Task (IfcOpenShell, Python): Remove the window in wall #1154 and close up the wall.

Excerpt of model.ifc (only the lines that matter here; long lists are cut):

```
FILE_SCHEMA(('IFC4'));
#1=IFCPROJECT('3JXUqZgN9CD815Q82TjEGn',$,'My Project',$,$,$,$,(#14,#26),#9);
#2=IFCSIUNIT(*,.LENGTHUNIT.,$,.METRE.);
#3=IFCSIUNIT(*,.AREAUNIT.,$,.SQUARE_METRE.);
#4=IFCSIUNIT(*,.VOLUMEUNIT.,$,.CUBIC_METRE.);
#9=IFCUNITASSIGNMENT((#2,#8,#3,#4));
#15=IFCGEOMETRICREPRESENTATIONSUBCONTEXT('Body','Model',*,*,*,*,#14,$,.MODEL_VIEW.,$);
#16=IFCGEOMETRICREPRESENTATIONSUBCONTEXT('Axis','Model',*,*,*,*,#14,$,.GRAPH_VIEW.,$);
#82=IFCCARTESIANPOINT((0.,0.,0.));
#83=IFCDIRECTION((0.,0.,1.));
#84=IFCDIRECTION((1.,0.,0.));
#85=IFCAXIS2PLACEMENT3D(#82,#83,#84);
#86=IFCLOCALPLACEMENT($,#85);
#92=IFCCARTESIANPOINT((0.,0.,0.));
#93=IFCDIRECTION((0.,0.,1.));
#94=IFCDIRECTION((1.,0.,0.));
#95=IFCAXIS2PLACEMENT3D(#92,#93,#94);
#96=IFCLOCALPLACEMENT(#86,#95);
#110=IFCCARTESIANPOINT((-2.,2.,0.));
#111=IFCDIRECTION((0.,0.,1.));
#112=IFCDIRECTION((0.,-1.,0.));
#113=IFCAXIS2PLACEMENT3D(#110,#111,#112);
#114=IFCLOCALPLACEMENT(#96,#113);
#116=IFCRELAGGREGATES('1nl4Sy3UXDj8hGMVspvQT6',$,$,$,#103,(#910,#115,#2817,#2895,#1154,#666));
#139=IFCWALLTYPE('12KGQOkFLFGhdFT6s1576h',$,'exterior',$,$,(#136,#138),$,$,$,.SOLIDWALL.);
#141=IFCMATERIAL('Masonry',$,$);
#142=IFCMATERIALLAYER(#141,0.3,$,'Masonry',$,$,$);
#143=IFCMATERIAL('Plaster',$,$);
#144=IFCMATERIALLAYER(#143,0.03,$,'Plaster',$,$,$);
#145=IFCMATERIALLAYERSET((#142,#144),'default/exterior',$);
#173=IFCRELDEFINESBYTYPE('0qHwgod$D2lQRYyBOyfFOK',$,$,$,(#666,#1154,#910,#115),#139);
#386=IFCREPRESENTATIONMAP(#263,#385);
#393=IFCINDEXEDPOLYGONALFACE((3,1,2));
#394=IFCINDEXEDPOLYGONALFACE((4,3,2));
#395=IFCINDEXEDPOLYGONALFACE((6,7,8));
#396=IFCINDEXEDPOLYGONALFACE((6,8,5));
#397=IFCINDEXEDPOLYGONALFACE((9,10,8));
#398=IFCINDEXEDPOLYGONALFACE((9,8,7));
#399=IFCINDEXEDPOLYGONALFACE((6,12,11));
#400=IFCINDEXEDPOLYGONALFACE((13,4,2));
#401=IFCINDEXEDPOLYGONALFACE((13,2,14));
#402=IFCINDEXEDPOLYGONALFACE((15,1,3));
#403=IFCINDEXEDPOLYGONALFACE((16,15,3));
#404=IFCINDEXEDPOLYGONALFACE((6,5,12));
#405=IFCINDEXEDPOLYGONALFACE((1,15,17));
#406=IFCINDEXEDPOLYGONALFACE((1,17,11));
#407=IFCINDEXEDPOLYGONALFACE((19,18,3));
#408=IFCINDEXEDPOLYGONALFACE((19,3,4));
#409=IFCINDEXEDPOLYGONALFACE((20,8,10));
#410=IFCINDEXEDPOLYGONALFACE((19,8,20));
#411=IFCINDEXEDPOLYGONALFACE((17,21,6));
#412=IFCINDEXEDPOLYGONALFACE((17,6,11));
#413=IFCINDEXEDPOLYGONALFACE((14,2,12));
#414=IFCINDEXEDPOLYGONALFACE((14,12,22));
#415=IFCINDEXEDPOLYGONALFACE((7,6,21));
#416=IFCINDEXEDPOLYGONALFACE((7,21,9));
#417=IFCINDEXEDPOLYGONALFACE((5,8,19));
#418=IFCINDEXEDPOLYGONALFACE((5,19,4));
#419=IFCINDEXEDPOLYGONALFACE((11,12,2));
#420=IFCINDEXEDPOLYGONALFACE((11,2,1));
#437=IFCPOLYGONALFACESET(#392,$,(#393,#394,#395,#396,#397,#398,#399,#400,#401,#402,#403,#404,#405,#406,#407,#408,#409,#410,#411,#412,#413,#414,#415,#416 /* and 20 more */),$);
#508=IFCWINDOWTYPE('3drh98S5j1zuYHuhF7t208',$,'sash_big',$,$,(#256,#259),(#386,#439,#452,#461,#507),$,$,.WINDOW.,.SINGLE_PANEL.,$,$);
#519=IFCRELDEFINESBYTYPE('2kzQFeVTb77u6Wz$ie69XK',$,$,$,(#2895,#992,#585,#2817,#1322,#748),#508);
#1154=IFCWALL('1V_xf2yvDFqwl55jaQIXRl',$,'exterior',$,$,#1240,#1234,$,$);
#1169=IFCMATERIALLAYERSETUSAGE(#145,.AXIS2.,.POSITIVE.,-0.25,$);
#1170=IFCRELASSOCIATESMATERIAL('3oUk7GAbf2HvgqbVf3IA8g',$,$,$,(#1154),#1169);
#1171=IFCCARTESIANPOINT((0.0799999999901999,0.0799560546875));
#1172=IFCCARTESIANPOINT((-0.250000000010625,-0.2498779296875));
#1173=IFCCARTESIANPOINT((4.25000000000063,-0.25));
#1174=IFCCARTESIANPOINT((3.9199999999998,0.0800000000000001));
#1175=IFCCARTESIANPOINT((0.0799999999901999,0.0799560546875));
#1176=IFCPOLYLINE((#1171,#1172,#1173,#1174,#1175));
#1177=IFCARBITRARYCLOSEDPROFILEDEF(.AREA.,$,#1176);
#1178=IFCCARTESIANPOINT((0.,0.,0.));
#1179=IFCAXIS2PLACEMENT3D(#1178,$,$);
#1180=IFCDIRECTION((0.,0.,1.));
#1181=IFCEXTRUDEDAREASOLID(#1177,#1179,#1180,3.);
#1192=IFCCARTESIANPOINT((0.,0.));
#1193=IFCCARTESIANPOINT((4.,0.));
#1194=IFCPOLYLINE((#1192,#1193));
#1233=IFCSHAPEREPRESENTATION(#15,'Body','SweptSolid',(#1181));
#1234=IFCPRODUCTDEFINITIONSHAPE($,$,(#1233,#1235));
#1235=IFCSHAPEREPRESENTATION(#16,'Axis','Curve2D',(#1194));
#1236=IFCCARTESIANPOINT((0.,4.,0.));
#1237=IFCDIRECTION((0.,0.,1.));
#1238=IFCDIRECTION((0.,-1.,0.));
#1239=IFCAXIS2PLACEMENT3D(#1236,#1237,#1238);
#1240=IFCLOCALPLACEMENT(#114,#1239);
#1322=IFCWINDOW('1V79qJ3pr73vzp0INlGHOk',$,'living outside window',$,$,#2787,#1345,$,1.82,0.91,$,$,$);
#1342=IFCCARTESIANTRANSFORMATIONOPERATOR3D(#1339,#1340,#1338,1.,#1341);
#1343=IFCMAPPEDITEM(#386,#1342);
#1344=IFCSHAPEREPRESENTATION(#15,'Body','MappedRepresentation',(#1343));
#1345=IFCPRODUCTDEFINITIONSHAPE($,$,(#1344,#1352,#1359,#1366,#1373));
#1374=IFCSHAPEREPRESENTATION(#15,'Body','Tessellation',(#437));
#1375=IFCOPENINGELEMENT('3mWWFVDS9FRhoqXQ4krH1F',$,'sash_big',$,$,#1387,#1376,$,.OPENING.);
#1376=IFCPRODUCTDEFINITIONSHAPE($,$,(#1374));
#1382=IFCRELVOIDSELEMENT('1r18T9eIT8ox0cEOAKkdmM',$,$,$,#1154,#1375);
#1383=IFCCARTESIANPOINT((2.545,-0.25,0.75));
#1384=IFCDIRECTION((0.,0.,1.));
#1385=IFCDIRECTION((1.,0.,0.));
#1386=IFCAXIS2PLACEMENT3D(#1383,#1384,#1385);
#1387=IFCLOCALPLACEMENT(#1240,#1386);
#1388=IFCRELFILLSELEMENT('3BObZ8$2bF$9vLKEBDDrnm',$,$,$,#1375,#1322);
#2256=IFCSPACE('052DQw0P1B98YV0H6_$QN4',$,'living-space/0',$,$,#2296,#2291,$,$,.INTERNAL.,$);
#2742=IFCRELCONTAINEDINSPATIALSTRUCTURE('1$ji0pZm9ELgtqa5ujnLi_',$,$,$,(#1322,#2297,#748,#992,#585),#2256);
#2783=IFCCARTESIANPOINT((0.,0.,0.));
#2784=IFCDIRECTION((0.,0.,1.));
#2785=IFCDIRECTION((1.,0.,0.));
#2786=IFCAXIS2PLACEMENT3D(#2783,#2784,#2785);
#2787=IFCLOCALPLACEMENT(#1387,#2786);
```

```python
import ifcopenshell
import ifcopenshell.api.feature
import ifcopenshell.api.root
import ifcopenshell.geom
import ifcopenshell.util.shape

model = ifcopenshell.open("model.ifc")
settings = ifcopenshell.geom.settings()


def volume(element):
    """Net volume in cubic metres, openings subtracted."""
    shape = ifcopenshell.geom.create_shape(settings, element)
    return ifcopenshell.util.shape.get_volume(shape.geometry)


window = model.by_guid("1V79qJ3pr73vzp0INlGHOk")
opening = window.FillsVoids[0].RelatingOpeningElement
wall = opening.VoidsElements[0].RelatingBuildingElement
before = volume(wall)

ifcopenshell.api.root.remove_product(model, product=window)
ifcopenshell.api.feature.remove_feature(model, feature=opening)

after = volume(wall)

print(f"wall volume {before:.3f} -> {after:.3f} m3")

model.write("model_rev.ifc")
```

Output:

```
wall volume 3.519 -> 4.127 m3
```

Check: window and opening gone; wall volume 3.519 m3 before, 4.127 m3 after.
